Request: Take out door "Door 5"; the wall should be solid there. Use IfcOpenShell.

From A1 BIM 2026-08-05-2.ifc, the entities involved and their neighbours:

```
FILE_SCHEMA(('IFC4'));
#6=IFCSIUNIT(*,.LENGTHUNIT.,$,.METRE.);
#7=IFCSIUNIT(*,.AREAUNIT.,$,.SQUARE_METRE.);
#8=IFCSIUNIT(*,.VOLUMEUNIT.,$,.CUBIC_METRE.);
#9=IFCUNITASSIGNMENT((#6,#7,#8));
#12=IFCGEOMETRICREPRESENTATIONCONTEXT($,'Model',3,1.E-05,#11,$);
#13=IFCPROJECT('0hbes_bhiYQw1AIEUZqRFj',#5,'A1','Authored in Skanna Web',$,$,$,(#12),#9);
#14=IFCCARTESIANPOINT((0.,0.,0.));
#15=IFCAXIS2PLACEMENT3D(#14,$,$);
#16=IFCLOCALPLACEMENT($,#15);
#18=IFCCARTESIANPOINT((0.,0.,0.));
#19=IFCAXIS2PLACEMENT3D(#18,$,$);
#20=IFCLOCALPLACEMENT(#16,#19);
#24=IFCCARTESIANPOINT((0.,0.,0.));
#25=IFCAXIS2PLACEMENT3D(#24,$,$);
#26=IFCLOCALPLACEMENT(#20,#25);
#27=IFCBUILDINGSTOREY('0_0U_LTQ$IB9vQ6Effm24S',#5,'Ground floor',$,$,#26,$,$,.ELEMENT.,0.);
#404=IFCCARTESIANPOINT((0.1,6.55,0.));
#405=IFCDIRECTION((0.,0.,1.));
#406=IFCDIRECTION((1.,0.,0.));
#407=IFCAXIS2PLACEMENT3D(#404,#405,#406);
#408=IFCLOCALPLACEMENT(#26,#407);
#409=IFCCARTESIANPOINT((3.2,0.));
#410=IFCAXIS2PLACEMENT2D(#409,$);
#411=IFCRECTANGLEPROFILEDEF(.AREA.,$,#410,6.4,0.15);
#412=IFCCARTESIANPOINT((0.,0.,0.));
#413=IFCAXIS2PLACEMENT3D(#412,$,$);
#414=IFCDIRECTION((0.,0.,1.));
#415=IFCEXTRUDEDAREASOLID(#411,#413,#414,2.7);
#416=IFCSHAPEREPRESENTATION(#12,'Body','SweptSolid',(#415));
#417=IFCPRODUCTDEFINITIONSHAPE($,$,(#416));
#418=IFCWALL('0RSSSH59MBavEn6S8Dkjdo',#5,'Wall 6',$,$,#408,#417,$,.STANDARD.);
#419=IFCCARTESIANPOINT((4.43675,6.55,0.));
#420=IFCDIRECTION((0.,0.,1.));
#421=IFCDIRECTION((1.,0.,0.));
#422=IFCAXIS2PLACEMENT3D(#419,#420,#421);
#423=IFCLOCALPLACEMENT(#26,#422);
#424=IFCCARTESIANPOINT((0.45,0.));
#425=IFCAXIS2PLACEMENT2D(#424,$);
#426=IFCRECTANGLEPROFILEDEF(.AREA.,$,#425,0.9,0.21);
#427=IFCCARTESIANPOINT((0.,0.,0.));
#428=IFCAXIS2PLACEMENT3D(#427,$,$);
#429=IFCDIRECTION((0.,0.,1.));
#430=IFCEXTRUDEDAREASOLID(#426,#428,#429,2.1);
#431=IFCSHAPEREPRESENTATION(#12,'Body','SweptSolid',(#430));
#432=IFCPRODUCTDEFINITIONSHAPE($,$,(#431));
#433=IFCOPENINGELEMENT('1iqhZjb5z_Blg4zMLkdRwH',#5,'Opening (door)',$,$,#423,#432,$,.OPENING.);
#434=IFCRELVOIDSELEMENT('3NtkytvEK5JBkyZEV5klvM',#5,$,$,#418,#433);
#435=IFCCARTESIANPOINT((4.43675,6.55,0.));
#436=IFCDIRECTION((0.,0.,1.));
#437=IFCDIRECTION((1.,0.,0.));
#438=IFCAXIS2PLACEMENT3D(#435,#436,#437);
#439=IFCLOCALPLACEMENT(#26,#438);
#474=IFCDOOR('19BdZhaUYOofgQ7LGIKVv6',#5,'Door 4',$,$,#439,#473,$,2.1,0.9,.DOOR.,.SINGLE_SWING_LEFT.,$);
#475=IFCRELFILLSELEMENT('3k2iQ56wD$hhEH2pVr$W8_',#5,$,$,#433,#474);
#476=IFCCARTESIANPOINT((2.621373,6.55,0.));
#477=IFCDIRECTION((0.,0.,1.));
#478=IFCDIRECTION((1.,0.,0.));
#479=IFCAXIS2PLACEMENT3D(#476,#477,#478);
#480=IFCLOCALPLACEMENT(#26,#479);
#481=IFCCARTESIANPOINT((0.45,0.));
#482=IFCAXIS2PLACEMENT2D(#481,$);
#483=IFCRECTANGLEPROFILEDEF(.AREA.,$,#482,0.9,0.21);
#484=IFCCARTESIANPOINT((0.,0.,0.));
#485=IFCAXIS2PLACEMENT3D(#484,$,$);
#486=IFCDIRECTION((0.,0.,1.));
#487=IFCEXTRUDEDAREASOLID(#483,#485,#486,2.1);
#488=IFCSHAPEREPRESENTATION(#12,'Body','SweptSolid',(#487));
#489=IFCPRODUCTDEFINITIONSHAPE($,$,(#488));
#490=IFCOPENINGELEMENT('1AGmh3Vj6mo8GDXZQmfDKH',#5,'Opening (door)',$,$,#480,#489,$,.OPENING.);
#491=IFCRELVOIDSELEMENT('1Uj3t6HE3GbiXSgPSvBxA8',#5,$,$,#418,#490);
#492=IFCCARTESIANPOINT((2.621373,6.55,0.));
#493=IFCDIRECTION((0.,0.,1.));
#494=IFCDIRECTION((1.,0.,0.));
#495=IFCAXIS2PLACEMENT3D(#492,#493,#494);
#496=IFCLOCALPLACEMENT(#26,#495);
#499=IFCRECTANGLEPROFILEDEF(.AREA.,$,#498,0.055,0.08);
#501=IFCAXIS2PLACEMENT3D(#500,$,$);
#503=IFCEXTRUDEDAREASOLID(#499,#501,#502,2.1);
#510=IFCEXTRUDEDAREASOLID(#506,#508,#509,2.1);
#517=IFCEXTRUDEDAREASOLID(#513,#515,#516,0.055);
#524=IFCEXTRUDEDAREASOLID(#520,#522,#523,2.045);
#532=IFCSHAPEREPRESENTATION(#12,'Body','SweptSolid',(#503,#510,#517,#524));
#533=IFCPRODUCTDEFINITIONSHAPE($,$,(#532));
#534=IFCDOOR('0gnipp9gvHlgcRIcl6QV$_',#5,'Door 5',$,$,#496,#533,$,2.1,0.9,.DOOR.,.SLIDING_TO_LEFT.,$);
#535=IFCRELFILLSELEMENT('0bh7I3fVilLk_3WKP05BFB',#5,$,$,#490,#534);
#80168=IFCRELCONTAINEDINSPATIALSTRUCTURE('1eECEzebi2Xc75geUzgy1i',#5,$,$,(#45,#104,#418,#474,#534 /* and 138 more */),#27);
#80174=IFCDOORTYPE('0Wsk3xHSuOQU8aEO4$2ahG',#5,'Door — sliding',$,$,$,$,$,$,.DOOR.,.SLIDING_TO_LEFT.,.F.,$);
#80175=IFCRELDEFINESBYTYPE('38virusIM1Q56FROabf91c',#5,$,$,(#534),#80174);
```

```python
import ifcopenshell
import ifcopenshell.api.feature
import ifcopenshell.api.root
import ifcopenshell.geom
import ifcopenshell.util.shape

model = ifcopenshell.open("A1 BIM 2026-08-05-2.ifc")
settings = ifcopenshell.geom.settings()


def volume(element):
    """Net volume in cubic metres, openings subtracted."""
    shape = ifcopenshell.geom.create_shape(settings, element)
    return ifcopenshell.util.shape.get_volume(shape.geometry)


door = model.by_guid("0gnipp9gvHlgcRIcl6QV$_")
opening = door.FillsVoids[0].RelatingOpeningElement
wall = opening.VoidsElements[0].RelatingBuildingElement
before = volume(wall)

ifcopenshell.api.root.remove_product(model, product=door)
ifcopenshell.api.feature.remove_feature(model, feature=opening)

after = volume(wall)

print(f"wall volume {before:.3f} -> {after:.3f} m3")

model.write("A1 BIM 2026-08-05-2_updated.ifc")
```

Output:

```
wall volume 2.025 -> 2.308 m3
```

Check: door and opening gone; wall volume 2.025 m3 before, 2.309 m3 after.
